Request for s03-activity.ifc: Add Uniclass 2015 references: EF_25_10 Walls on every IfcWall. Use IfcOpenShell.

First a look at what the model holds.

```python
import ifcopenshell

model = ifcopenshell.open("s03-activity.ifc")
print(model.schema)
print("classifications:", [c.Name for c in model.by_type("IfcClassification")])
for ifc_class in ("IfcDoor", "IfcRoof", "IfcStair", "IfcWall", "IfcWindow"):
    print(ifc_class, len(model.by_type(ifc_class)))
```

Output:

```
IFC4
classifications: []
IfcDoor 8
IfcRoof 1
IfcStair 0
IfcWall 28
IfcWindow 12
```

```python
import ifcopenshell
import ifcopenshell.api.classification

model = ifcopenshell.open("s03-activity.ifc")

system = ifcopenshell.api.classification.add_classification(model, classification="Uniclass 2015")

codes = {
    "IfcWall": ("EF_25_10", "Walls"),
}
for ifc_class, (code, name) in codes.items():
    products = model.by_type(ifc_class)
    ifcopenshell.api.classification.add_reference(
        model, products=products, classification=system, identification=code, name=name
    )
    print(code, len(products))

model.write("s03-activity-out.ifc")
```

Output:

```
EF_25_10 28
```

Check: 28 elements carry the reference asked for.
